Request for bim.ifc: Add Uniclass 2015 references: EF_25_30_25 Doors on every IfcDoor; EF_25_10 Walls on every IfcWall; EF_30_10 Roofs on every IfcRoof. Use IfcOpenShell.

First a look at what the model holds.

```python
import ifcopenshell

model = ifcopenshell.open("bim.ifc")
print(model.schema)
print("classifications:", [c.Name for c in model.by_type("IfcClassification")])
for ifc_class in ("IfcDoor", "IfcRoof", "IfcStair", "IfcWall", "IfcWindow"):
    print(ifc_class, len(model.by_type(ifc_class)))
```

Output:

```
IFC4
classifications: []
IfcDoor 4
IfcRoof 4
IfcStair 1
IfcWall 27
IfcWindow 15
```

```python
import ifcopenshell
import ifcopenshell.api.classification

model = ifcopenshell.open("bim.ifc")

system = ifcopenshell.api.classification.add_classification(model, classification="Uniclass 2015")

codes = {
    "IfcDoor": ("EF_25_30_25", "Doors"),
    "IfcWall": ("EF_25_10", "Walls"),
    "IfcRoof": ("EF_30_10", "Roofs"),
}
for ifc_class, (code, name) in codes.items():
    products = model.by_type(ifc_class)
    ifcopenshell.api.classification.add_reference(
        model, products=products, classification=system, identification=code, name=name
    )
    print(code, len(products))

model.write("bim_updated.ifc")
```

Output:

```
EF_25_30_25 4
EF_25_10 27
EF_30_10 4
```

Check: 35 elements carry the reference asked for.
